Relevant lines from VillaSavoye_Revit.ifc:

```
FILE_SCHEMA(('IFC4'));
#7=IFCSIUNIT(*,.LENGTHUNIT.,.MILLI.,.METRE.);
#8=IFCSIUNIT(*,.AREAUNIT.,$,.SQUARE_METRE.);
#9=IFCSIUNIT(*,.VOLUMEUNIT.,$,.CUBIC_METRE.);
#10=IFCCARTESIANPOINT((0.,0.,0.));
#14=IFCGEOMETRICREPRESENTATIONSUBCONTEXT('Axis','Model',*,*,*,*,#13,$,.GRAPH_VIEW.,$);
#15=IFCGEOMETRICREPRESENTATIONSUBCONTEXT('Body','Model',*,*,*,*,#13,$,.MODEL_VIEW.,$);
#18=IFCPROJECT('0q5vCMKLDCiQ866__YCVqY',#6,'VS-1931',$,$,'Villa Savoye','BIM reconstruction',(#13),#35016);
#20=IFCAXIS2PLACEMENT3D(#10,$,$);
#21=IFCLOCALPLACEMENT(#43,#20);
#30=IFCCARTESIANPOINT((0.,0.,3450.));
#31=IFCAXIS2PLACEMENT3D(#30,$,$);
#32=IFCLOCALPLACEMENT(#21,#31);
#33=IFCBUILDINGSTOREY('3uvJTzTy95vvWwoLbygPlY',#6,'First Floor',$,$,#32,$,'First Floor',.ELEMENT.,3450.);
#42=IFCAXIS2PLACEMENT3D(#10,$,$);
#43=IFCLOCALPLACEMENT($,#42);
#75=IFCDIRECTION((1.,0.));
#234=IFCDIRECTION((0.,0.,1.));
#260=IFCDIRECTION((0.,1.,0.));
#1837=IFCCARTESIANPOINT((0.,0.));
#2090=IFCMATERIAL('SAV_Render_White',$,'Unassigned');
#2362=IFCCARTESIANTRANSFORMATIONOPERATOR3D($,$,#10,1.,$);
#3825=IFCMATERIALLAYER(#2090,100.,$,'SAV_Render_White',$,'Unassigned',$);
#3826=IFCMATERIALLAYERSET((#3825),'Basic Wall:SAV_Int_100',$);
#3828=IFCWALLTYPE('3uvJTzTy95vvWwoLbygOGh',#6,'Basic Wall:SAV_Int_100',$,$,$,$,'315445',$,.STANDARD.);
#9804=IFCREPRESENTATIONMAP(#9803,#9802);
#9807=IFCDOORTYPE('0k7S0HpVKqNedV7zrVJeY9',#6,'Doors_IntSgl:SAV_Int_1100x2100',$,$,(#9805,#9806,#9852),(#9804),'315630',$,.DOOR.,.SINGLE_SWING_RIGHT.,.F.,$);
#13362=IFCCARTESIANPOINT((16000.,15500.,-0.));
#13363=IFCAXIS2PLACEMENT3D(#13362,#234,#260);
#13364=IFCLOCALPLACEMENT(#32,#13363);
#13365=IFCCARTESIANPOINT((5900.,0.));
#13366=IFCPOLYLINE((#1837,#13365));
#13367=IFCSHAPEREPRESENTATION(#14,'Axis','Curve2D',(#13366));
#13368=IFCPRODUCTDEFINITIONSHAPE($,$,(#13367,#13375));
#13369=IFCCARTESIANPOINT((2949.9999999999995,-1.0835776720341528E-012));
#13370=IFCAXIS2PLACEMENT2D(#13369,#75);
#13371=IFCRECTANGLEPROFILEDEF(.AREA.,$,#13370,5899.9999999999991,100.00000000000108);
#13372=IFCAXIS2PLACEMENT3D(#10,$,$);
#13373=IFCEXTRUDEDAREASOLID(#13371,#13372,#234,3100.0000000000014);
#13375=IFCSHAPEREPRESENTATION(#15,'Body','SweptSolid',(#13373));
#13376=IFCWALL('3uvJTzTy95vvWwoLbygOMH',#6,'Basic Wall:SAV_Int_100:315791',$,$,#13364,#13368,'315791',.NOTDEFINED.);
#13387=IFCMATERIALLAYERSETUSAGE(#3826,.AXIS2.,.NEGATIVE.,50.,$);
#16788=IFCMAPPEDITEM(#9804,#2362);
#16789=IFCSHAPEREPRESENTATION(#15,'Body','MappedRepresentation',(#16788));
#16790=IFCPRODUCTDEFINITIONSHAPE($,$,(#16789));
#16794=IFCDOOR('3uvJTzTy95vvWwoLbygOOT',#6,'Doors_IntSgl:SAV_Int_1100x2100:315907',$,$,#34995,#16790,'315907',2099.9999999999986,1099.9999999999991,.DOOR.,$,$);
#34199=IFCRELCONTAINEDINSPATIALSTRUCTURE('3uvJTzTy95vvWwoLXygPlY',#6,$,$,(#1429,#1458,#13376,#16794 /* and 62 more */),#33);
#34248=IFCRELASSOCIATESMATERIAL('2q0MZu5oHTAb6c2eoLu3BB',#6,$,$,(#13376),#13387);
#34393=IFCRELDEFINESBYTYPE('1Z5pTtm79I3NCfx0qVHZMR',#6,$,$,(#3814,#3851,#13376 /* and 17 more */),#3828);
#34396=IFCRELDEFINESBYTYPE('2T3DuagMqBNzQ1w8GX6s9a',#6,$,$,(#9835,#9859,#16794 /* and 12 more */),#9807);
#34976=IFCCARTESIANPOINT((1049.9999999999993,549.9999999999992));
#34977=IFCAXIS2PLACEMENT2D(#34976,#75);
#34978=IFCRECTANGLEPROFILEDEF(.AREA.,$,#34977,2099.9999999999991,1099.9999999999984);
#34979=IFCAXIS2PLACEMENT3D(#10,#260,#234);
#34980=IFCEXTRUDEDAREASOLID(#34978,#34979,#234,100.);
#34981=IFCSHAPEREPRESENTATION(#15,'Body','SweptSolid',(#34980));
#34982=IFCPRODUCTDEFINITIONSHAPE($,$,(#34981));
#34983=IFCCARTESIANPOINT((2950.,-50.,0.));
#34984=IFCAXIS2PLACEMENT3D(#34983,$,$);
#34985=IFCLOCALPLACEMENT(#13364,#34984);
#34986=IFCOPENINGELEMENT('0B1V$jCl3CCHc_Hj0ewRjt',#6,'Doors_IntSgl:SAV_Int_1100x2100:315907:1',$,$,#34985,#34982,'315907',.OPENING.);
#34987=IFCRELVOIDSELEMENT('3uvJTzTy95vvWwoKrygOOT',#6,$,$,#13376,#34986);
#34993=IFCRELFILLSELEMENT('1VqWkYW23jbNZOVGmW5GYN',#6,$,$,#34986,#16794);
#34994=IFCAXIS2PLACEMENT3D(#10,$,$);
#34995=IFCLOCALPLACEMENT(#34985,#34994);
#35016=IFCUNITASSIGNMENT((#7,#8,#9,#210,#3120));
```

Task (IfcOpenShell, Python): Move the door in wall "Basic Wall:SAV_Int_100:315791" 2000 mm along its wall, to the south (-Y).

```python
import ifcopenshell
import ifcopenshell.api.geometry
import ifcopenshell.util.placement

model = ifcopenshell.open("VillaSavoye_Revit.ifc")

door = model.by_id(16794)
opening = door.FillsVoids[0].RelatingOpeningElement
wall = opening.VoidsElements[0].RelatingBuildingElement

wall_matrix = ifcopenshell.util.placement.get_local_placement(wall.ObjectPlacement)
shift = wall_matrix[:3, 0] * -2000.0
before = ifcopenshell.util.placement.get_local_placement(door.ObjectPlacement)[:3, 3].copy()

# The door is placed relative to its opening, so it follows when the opening moves.
matrix = ifcopenshell.util.placement.get_local_placement(opening.ObjectPlacement)
matrix[:3, 3] += shift
ifcopenshell.api.geometry.edit_object_placement(
    model, product=opening, matrix=matrix, is_si=False, should_transform_children=True
)

after = ifcopenshell.util.placement.get_local_placement(door.ObjectPlacement)[:3, 3]
print("door moved by", (after - before).round(3) + 0.0)

model.write("VillaSavoye_Revit-out.ifc")
```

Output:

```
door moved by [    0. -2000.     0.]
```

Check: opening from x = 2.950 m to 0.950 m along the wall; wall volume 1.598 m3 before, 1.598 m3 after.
